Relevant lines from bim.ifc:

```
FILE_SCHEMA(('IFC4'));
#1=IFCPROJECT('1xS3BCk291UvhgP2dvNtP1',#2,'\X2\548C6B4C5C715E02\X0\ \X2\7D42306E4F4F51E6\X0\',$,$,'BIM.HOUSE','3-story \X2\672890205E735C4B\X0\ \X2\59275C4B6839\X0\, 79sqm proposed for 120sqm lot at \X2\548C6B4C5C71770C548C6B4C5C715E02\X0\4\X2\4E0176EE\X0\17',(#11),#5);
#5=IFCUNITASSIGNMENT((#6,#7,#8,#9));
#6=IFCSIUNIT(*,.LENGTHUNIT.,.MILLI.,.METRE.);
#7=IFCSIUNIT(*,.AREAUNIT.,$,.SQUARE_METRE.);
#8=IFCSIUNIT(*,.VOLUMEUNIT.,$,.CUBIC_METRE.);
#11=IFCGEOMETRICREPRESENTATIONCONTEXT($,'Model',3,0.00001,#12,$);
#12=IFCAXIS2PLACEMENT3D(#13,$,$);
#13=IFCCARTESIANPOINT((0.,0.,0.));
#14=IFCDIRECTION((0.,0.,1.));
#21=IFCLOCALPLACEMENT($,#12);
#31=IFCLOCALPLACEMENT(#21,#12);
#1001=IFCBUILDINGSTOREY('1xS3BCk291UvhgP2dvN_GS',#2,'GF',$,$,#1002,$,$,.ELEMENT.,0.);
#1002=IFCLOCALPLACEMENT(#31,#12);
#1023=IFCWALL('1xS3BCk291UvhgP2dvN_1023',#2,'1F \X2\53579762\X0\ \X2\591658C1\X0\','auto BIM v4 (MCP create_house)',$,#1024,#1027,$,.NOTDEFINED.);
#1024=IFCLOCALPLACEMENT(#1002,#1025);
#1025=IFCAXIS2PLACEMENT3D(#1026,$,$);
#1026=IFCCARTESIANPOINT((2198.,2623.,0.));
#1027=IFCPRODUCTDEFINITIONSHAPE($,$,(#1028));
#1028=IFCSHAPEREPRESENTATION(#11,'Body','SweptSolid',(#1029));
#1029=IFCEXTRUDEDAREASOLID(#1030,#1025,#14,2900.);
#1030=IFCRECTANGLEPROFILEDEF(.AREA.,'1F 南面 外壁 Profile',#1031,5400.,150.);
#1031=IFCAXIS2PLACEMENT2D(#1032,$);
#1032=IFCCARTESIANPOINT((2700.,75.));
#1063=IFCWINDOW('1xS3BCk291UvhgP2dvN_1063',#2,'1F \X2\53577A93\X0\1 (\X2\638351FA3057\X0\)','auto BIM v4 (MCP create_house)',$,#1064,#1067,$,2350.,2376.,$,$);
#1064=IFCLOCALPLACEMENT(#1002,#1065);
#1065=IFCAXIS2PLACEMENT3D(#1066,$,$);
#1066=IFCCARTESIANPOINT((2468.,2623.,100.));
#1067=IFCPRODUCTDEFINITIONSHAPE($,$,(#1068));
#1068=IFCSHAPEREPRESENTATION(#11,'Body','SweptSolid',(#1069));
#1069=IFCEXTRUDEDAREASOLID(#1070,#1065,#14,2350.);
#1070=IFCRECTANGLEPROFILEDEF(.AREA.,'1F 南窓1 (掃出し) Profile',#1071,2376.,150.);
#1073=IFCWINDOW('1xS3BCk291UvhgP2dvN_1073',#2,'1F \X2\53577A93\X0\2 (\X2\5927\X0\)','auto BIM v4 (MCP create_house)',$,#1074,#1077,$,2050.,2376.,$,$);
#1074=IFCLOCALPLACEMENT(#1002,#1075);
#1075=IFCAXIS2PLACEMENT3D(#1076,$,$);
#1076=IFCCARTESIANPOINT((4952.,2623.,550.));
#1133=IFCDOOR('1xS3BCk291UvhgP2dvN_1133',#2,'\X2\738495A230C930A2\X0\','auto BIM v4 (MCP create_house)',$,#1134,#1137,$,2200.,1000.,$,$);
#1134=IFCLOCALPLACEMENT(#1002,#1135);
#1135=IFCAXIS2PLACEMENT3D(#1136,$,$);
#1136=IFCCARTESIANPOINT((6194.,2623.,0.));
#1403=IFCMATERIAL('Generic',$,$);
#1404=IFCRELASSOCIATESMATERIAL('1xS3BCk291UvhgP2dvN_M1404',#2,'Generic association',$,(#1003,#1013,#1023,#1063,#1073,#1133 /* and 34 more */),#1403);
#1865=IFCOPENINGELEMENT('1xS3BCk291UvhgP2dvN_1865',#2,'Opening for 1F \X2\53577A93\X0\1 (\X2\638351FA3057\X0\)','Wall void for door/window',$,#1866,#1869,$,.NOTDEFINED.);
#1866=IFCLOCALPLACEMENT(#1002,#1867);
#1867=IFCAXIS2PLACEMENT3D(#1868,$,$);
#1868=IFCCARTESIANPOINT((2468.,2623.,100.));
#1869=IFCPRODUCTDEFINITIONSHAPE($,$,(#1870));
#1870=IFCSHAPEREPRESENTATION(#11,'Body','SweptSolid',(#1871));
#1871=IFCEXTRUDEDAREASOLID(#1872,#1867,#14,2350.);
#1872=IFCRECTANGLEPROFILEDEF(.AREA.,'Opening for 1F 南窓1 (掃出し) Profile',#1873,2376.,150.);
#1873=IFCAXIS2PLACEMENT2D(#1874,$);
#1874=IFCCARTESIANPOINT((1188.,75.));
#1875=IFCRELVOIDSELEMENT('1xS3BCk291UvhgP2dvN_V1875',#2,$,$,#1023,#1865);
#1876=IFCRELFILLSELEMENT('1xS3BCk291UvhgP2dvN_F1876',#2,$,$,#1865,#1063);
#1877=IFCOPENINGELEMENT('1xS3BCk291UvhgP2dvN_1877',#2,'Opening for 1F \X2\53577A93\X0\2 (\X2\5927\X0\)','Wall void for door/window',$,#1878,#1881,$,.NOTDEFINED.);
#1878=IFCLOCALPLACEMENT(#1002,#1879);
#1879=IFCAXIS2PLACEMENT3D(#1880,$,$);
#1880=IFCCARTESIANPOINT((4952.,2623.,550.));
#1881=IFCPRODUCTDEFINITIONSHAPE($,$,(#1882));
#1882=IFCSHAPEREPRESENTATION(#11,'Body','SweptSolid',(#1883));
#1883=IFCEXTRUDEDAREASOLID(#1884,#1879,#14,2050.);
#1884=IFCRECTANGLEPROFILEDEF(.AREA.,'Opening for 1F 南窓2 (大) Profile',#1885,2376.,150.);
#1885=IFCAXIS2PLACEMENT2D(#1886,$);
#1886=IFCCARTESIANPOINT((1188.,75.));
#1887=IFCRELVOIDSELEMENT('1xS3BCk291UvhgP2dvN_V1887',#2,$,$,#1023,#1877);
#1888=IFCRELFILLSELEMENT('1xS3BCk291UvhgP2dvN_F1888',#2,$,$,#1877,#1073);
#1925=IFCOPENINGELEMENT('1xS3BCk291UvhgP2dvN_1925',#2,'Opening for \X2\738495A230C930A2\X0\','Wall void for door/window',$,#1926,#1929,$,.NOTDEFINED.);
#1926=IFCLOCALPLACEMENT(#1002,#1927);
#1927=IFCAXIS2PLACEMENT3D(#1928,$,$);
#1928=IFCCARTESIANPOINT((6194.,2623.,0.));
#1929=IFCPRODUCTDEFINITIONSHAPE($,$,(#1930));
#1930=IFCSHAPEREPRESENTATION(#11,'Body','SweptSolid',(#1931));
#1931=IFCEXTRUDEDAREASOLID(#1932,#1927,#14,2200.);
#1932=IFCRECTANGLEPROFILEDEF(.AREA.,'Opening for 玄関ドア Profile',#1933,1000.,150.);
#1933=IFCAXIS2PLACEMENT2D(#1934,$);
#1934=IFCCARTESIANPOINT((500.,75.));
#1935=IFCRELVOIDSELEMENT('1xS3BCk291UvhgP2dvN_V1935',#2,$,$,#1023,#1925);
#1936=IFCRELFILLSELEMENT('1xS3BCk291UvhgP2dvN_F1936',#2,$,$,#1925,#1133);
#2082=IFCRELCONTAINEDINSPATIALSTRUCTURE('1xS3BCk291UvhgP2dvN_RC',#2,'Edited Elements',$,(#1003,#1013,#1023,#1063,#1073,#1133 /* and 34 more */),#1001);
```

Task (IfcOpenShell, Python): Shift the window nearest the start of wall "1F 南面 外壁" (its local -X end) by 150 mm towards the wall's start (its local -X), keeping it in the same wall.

```python
import ifcopenshell
import ifcopenshell.api.geometry
import ifcopenshell.util.placement
import ifcopenshell.util.unit

model = ifcopenshell.open("bim.ifc")
unit_scale = ifcopenshell.util.unit.calculate_unit_scale(model)

window = model.by_guid("1xS3BCk291UvhgP2dvN_1063")
opening = window.FillsVoids[0].RelatingOpeningElement
wall = opening.VoidsElements[0].RelatingBuildingElement

wall_matrix = ifcopenshell.util.placement.get_local_placement(wall.ObjectPlacement)
shift = wall_matrix[:3, 0] * -0.15 / unit_scale
before = ifcopenshell.util.placement.get_local_placement(window.ObjectPlacement)[:3, 3].copy()

# The window is not placed relative to its opening, so move both.
for product in (opening, window):
    matrix = ifcopenshell.util.placement.get_local_placement(product.ObjectPlacement)
    matrix[:3, 3] += shift
    ifcopenshell.api.geometry.edit_object_placement(model, product=product, matrix=matrix, is_si=False)

after = ifcopenshell.util.placement.get_local_placement(window.ObjectPlacement)[:3, 3]
print("window moved by", (after - before).round(3) + 0.0)

model.write("bim_v2.ifc")
```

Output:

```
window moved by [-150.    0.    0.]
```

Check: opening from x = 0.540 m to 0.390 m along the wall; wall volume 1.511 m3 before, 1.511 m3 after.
